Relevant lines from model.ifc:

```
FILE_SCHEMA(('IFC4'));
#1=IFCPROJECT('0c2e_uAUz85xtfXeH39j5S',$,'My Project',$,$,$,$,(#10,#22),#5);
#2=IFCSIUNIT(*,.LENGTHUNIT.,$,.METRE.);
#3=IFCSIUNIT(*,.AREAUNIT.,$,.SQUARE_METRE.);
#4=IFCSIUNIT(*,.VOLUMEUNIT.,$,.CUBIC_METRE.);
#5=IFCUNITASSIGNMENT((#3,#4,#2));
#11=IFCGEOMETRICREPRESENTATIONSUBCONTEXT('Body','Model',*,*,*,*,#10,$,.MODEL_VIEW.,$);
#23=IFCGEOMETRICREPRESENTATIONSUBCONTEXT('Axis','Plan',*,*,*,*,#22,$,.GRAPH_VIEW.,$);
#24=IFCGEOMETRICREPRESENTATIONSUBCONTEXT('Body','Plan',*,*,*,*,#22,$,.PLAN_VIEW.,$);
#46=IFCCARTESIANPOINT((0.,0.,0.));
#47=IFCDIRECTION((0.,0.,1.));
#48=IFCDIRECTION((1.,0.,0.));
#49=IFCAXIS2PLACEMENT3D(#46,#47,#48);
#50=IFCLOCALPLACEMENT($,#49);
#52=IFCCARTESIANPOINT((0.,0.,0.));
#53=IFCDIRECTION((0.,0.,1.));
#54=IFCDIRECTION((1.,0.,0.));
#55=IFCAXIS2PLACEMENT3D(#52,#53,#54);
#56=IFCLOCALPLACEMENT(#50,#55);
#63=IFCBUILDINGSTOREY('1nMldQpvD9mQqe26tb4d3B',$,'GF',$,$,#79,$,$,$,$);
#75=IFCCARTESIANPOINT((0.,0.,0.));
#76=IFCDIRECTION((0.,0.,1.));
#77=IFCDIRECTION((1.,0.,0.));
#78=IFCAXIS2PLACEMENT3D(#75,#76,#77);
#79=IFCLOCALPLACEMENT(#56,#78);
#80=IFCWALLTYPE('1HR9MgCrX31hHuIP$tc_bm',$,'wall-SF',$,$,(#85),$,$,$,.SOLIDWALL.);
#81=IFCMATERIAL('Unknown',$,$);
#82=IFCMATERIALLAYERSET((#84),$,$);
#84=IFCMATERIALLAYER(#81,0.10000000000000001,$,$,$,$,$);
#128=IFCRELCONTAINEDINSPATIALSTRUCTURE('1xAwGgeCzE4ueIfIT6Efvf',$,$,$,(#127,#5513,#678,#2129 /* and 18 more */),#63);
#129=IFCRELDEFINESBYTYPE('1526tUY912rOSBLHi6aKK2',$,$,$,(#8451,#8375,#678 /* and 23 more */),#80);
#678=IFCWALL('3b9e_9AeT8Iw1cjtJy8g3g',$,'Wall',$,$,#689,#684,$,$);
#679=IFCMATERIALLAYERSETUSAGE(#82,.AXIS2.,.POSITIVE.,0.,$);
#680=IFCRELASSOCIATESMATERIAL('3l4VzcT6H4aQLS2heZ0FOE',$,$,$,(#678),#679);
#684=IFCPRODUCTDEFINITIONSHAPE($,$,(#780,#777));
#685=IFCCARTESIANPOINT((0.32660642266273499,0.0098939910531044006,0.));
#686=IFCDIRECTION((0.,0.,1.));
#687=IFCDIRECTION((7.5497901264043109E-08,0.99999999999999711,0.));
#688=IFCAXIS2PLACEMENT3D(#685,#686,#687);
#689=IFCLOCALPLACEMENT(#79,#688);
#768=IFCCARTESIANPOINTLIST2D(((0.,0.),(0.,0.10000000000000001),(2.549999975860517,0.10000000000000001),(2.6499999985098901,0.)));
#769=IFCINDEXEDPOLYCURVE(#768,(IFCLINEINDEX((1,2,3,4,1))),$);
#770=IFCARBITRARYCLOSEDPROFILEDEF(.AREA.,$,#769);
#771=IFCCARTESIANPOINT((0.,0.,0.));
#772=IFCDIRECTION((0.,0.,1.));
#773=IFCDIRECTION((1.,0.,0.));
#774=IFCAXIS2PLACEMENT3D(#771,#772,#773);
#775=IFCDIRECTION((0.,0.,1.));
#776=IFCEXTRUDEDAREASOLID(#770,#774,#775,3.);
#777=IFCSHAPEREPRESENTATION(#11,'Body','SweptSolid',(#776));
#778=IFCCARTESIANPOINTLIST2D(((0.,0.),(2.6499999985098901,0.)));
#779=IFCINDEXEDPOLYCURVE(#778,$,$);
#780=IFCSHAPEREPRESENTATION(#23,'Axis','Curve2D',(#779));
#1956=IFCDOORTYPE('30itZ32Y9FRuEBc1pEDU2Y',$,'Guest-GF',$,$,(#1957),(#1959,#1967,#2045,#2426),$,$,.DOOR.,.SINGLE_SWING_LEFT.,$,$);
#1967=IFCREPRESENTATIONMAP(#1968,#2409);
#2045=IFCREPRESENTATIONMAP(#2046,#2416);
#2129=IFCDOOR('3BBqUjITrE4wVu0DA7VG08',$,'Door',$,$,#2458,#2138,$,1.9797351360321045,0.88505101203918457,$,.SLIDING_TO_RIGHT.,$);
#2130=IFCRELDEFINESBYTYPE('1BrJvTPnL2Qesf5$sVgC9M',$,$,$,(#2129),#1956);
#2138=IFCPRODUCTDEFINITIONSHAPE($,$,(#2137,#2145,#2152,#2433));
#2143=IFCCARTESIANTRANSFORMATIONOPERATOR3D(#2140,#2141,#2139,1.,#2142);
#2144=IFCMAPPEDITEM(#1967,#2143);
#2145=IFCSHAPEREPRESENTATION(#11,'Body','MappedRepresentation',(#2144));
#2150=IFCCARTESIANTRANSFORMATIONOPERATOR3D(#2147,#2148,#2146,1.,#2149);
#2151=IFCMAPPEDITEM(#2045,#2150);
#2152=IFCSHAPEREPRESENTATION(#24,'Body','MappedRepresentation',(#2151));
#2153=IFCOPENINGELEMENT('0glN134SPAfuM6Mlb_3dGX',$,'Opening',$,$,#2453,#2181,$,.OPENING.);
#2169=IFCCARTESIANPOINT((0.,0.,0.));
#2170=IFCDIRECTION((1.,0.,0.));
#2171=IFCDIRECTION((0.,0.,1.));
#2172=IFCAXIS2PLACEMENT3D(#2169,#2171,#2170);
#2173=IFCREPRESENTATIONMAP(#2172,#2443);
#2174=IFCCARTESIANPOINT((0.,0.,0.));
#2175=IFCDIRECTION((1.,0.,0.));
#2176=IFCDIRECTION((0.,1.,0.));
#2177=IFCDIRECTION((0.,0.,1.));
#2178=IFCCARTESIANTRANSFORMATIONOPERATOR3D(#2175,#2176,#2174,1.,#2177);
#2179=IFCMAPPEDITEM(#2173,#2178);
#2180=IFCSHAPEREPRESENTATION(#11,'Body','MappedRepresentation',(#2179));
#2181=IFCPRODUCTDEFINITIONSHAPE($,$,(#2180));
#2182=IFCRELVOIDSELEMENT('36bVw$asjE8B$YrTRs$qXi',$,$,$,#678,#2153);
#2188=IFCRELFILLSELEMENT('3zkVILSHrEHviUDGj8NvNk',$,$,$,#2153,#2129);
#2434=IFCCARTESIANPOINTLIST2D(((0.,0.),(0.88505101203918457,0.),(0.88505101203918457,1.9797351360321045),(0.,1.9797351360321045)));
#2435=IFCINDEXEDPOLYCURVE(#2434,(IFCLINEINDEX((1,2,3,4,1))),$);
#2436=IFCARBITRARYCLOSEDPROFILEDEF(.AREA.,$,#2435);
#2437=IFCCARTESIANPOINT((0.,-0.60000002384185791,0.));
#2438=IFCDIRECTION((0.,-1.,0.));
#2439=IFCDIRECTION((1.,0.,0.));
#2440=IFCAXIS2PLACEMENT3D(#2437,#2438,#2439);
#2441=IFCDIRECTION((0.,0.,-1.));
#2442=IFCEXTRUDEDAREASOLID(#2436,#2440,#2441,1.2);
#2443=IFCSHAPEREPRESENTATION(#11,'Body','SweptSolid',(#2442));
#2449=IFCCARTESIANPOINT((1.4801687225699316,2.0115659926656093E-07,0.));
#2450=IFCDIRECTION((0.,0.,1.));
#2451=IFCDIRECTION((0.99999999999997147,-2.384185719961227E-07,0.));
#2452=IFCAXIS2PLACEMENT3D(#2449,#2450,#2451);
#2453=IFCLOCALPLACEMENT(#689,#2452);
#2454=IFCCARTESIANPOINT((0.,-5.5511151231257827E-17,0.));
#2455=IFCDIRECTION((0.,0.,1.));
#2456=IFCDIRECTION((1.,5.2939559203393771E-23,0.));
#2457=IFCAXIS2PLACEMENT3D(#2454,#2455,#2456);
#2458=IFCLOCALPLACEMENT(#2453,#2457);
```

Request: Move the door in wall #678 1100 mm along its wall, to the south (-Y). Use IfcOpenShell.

```python
import ifcopenshell
import ifcopenshell.api.geometry
import ifcopenshell.util.placement
import ifcopenshell.util.unit

model = ifcopenshell.open("model.ifc")
unit_scale = ifcopenshell.util.unit.calculate_unit_scale(model)

door = model.by_guid("3BBqUjITrE4wVu0DA7VG08")
opening = door.FillsVoids[0].RelatingOpeningElement
wall = opening.VoidsElements[0].RelatingBuildingElement

wall_matrix = ifcopenshell.util.placement.get_local_placement(wall.ObjectPlacement)
shift = wall_matrix[:3, 0] * -1.1 / unit_scale
before = ifcopenshell.util.placement.get_local_placement(door.ObjectPlacement)[:3, 3].copy()

# The door is placed relative to its opening, so it follows when the opening moves.
matrix = ifcopenshell.util.placement.get_local_placement(opening.ObjectPlacement)
matrix[:3, 3] += shift
ifcopenshell.api.geometry.edit_object_placement(
    model, product=opening, matrix=matrix, is_si=False, should_transform_children=True
)

after = ifcopenshell.util.placement.get_local_placement(door.ObjectPlacement)[:3, 3]
print("door moved by", (after - before).round(3) + 0.0)

model.write("model_updated.ifc")
```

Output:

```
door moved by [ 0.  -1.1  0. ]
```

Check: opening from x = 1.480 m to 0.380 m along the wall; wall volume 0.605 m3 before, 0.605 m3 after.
